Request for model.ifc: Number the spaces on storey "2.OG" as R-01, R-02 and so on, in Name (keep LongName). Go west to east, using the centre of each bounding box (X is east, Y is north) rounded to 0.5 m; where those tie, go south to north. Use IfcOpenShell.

First a look at what the model holds.

```python
import ifcopenshell
import ifcopenshell.util.element
import ifcopenshell.util.placement

model = ifcopenshell.open("model.ifc")
print(model.schema)
storey = next(s for s in model.by_type("IfcBuildingStorey") if s.Name == "2.OG")
spaces = [e for e in ifcopenshell.util.element.get_decomposition(storey) if e.is_a("IfcSpace")]
for e in sorted(spaces, key=lambda e: e.id()):
    origin = ifcopenshell.util.placement.get_local_placement(e.ObjectPlacement)[:3, 3]
    print(e.id(), e.Name, e.LongName, origin.round(2) + 0.0, sep=" | ")
```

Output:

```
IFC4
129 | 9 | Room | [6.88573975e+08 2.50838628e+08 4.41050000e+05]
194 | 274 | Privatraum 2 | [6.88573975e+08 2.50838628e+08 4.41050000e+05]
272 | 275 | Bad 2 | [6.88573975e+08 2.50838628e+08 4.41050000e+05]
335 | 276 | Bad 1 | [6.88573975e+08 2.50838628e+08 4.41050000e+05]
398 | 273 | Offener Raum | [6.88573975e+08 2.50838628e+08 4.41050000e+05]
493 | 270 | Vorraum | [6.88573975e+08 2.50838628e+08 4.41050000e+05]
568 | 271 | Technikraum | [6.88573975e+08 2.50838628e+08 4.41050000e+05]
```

```python
import ifcopenshell
import ifcopenshell.geom
import ifcopenshell.util.element
import ifcopenshell.util.shape

model = ifcopenshell.open("model.ifc")
settings = ifcopenshell.geom.settings()
settings.set("use-world-coords", True)


def centre(element):
    shape = ifcopenshell.geom.create_shape(settings, element)
    return ifcopenshell.util.shape.get_bbox_centroid(shape.geometry)


storey = next(s for s in model.by_type("IfcBuildingStorey") if s.Name == "2.OG")
spaces = [e for e in ifcopenshell.util.element.get_decomposition(storey) if e.is_a("IfcSpace")]

# Insertion points can sit at a corner or the storey origin, so sort by the geometry (in metres).
centres = {e: centre(e) for e in spaces}
spaces.sort(key=lambda e: (round(centres[e][0] / 0.5), centres[e][1]))

for i, e in enumerate(spaces, start=1):
    number = f"R-{i:02d}"
    e.Name = number
    print(e.id(), number)

model.write("model_rev.ifc")
```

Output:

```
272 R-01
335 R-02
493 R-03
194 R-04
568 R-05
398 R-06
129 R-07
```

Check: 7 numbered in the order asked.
